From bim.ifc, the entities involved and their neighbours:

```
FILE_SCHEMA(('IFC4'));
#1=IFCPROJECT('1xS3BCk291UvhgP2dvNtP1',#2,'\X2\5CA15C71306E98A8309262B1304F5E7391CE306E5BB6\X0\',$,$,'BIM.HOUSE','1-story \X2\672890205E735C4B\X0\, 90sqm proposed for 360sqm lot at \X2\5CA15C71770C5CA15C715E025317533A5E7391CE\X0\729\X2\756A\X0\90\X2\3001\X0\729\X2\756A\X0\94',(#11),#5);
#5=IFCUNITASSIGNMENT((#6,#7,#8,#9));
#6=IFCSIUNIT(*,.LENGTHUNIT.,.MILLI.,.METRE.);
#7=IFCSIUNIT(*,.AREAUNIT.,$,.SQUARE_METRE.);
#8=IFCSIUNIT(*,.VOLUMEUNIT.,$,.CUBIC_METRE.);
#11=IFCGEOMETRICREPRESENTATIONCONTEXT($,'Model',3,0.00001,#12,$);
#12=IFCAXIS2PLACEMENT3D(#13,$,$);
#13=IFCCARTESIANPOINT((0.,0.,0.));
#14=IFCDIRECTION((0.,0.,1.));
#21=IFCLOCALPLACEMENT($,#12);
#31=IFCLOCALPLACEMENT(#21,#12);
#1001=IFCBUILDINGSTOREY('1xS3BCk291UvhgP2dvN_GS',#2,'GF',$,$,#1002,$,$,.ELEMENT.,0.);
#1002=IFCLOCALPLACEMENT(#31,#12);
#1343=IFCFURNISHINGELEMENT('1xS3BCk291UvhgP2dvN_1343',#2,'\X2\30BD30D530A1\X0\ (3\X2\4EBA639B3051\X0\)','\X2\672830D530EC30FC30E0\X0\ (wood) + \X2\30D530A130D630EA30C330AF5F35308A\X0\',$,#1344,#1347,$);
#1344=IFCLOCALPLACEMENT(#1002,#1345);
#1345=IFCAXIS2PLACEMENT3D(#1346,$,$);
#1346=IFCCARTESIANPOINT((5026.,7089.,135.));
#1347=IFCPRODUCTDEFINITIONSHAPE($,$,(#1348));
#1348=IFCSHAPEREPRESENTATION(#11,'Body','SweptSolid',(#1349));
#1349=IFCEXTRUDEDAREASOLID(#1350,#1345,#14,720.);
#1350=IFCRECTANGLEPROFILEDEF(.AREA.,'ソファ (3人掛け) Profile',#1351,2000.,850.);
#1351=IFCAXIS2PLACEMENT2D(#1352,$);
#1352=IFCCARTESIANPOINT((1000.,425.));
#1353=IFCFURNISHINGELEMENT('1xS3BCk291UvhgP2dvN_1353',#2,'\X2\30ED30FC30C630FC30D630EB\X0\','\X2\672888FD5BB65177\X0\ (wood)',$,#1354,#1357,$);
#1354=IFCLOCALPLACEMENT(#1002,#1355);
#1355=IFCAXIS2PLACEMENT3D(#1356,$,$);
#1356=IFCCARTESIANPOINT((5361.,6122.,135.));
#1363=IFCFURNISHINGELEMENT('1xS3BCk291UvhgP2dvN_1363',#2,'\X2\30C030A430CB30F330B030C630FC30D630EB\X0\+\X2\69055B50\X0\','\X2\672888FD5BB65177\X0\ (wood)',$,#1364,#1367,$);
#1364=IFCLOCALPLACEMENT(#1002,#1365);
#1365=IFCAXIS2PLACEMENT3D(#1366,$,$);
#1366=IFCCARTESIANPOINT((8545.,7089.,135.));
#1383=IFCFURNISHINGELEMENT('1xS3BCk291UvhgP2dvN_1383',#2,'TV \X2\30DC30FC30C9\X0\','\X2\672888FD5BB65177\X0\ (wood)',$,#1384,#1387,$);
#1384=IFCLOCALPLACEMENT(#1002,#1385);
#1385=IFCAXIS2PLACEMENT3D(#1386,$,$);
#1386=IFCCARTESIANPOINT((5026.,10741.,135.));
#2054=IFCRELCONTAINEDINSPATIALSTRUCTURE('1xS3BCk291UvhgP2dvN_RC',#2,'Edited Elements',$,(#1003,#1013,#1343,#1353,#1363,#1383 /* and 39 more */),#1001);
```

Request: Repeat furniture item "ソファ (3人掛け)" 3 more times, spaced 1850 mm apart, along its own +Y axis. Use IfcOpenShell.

```python
import ifcopenshell
import ifcopenshell.api.geometry
import ifcopenshell.api.root
import ifcopenshell.util.element
import ifcopenshell.util.placement
import ifcopenshell.util.unit

model = ifcopenshell.open("bim.ifc")
unit_scale = ifcopenshell.util.unit.calculate_unit_scale(model)


def reuse_history(source, copy):
    """copy_class also copies each property set's owner history, people and application; keep the originals."""
    for rel in copy.IsDefinedBy:
        if rel.is_a("IfcRelDefinesByProperties") and (history := rel.RelatingPropertyDefinition.OwnerHistory):
            rel.RelatingPropertyDefinition.OwnerHistory = source.OwnerHistory
            ifcopenshell.util.element.remove_deep2(model, history)


source = model.by_guid("1xS3BCk291UvhgP2dvN_1343")
base = ifcopenshell.util.placement.get_local_placement(source.ObjectPlacement)
step = base[:3, 1] * 1.85 / unit_scale

for i in range(1, 4):
    copy = ifcopenshell.api.root.copy_class(model, product=source)
    copy.Representation = ifcopenshell.util.element.copy_deep(
        model, source.Representation, exclude=["IfcGeometricRepresentationContext", "IfcRepresentationMap"]
    )
    reuse_history(source, copy)
    matrix = base.copy()
    matrix[:3, 3] += i * step
    print("added at", matrix[:3, 3].round(3) + 0.0)
    ifcopenshell.api.geometry.edit_object_placement(model, product=copy, matrix=matrix, is_si=False)

model.write("bim-out.ifc")
```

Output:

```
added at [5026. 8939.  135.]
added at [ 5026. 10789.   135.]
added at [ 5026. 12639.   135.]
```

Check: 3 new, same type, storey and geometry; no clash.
